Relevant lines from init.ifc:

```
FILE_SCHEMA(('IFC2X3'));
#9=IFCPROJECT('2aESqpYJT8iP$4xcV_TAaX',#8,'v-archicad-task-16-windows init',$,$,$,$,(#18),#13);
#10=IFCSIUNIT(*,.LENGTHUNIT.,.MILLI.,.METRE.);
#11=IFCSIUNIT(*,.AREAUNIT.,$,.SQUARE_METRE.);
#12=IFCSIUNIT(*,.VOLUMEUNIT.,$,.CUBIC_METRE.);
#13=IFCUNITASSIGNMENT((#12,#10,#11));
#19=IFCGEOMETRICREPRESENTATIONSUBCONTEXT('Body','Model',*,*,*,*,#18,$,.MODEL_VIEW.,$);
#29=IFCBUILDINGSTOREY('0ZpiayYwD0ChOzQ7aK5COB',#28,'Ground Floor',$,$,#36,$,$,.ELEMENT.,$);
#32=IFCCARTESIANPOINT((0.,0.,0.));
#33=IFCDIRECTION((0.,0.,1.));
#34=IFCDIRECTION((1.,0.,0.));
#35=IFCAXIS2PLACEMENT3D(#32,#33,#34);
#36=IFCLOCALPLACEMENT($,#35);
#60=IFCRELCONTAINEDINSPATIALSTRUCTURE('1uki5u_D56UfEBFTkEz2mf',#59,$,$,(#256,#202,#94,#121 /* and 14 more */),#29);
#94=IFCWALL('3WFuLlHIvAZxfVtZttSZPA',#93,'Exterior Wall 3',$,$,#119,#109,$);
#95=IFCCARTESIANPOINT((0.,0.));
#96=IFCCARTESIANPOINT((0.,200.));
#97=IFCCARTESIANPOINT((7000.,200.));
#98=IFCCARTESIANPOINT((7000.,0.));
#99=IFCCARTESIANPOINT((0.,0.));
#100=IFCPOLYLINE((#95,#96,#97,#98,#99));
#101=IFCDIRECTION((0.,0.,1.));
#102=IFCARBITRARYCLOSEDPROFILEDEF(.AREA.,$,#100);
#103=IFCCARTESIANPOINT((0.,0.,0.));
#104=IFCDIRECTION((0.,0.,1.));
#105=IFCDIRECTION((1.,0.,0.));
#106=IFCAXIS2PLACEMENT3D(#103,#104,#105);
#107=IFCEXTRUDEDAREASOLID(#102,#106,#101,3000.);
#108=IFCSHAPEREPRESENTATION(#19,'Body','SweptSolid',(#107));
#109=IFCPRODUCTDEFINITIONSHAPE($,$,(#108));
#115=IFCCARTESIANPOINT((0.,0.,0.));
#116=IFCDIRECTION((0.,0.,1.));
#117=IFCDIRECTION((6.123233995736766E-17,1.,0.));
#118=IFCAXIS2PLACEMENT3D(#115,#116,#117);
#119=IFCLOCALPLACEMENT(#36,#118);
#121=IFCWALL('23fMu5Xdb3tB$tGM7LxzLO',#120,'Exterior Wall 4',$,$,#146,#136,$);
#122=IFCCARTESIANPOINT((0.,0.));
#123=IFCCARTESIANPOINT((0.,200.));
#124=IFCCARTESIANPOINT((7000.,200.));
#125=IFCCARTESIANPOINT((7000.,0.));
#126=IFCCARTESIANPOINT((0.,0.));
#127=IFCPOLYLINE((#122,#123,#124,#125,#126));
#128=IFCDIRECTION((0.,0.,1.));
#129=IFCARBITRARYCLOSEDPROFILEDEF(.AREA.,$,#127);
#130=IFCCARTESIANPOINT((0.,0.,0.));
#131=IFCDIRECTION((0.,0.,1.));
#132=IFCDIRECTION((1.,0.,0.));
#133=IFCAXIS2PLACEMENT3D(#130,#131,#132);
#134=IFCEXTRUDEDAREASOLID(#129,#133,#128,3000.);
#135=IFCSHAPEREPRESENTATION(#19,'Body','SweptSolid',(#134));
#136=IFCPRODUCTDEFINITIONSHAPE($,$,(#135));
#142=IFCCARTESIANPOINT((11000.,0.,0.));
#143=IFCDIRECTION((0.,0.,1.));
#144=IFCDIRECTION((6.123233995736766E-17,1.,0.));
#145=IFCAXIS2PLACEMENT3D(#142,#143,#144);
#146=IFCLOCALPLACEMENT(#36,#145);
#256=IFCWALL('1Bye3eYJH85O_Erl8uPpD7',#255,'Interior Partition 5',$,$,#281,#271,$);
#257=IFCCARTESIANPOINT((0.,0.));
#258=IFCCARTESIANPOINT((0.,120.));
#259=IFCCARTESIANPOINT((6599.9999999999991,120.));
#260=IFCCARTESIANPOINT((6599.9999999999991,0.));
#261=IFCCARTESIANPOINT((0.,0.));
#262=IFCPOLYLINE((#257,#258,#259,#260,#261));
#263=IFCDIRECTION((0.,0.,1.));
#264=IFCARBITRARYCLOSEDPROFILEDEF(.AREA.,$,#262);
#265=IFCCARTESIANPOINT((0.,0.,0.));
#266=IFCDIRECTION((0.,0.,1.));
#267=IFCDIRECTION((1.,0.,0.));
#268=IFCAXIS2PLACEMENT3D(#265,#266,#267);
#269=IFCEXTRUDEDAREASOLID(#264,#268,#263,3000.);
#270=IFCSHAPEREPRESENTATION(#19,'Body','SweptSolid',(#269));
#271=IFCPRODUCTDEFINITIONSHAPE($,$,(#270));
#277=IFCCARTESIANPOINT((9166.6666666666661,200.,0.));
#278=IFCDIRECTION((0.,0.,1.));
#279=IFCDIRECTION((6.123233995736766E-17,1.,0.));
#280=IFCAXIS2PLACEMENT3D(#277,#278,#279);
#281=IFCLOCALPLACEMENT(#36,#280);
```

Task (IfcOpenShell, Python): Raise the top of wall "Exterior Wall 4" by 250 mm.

```python
import ifcopenshell
import ifcopenshell.geom
import ifcopenshell.util.representation
import ifcopenshell.util.shape
import ifcopenshell.util.unit

model = ifcopenshell.open("init.ifc")
unit_scale = ifcopenshell.util.unit.calculate_unit_scale(model)
settings = ifcopenshell.geom.settings()


def volume(element):
    """Net volume in cubic metres, openings subtracted."""
    shape = ifcopenshell.geom.create_shape(settings, element)
    return ifcopenshell.util.shape.get_volume(shape.geometry)


wall = model.by_id(121)
before = volume(wall)

body = ifcopenshell.util.representation.get_representation(wall, "Model", "Body")
solid = body.Items[0]
old_height = solid.Depth
solid.Depth += 0.25 / unit_scale
after = volume(wall)

print(f"height {old_height:g} -> {solid.Depth:g}, volume {before:.3f} -> {after:.3f} m3")

model.write("init-out.ifc")
```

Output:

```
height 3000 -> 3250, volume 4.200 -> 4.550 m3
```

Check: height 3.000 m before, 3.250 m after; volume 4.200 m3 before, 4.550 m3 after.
